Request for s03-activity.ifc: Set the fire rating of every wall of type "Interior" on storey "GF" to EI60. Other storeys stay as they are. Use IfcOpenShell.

First a look at what the model holds.

```python
import ifcopenshell
import ifcopenshell.util.element

model = ifcopenshell.open("s03-activity.ifc")
print(model.schema)
storey = next(s for s in model.by_type("IfcBuildingStorey") if s.Name == "GF")
walls = [e for e in ifcopenshell.util.element.get_decomposition(storey) if e.is_a("IfcWall")]
seen = {}
for e in walls:
    element_type = ifcopenshell.util.element.get_type(e)
    key = (element_type.Name if element_type != e and element_type else None, ifcopenshell.util.element.get_pset(e, "Pset_WallCommon", "FireRating"))
    seen[key] = seen.get(key, 0) + 1
for (name, value), count in sorted(seen.items(), key=str):
    print(count, "x", name, "|", value)
```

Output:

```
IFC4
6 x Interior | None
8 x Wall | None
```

```python
import ifcopenshell
import ifcopenshell.api.pset
import ifcopenshell.util.element

model = ifcopenshell.open("s03-activity.ifc")

storey = next(s for s in model.by_type("IfcBuildingStorey") if s.Name == "GF")
walls = [e for e in ifcopenshell.util.element.get_decomposition(storey) if e.is_a("IfcWall")]

count = 0
for e in walls:
    element_type = ifcopenshell.util.element.get_type(e)
    if element_type in (None, e) or element_type.Name != "Interior":
        continue
    # add_pset returns the element's existing set when there is one.
    pset = ifcopenshell.api.pset.add_pset(model, product=e, name="Pset_WallCommon")
    ifcopenshell.api.pset.edit_pset(model, pset=pset, properties={"FireRating": "EI60"})
    count += 1

print(count, "walls updated")

model.write("s03-activity_updated.ifc")
```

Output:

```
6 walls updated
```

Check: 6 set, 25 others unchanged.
